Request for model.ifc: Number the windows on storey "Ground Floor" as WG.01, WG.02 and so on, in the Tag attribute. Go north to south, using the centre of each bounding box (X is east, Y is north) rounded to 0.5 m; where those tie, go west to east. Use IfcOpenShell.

First a look at what the model holds.

```python
import ifcopenshell
import ifcopenshell.util.element
import ifcopenshell.util.placement

model = ifcopenshell.open("model.ifc")
print(model.schema)
storey = next(s for s in model.by_type("IfcBuildingStorey") if s.Name == "Ground Floor")
windows = [e for e in ifcopenshell.util.element.get_decomposition(storey) if e.is_a("IfcWindow")]
for e in sorted(windows, key=lambda e: e.id()):
    origin = ifcopenshell.util.placement.get_local_placement(e.ObjectPlacement)[:3, 3]
    print(e.id(), e.Tag, e.Name, origin.round(2) + 0.0, sep=" | ")
```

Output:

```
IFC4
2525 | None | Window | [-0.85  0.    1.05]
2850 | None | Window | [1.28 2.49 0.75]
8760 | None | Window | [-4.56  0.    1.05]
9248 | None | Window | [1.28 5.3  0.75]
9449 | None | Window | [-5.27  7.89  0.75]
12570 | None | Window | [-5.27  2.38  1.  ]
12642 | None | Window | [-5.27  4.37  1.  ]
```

```python
import ifcopenshell
import ifcopenshell.geom
import ifcopenshell.util.element
import ifcopenshell.util.shape

model = ifcopenshell.open("model.ifc")
settings = ifcopenshell.geom.settings()
settings.set("use-world-coords", True)


def centre(element):
    shape = ifcopenshell.geom.create_shape(settings, element)
    return ifcopenshell.util.shape.get_bbox_centroid(shape.geometry)


storey = next(s for s in model.by_type("IfcBuildingStorey") if s.Name == "Ground Floor")
windows = [e for e in ifcopenshell.util.element.get_decomposition(storey) if e.is_a("IfcWindow")]

# Insertion points can sit at a corner or the storey origin, so sort by the geometry (in metres).
centres = {e: centre(e) for e in windows}
windows.sort(key=lambda e: (-round(centres[e][1] / 0.5), centres[e][0]))

for i, e in enumerate(windows, start=1):
    number = f"WG.{i:02d}"
    e.Tag = number
    print(e.id(), number)

model.write("model_rev.ifc")
```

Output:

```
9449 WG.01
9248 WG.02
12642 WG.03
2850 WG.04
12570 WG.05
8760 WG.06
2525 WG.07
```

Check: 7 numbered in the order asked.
